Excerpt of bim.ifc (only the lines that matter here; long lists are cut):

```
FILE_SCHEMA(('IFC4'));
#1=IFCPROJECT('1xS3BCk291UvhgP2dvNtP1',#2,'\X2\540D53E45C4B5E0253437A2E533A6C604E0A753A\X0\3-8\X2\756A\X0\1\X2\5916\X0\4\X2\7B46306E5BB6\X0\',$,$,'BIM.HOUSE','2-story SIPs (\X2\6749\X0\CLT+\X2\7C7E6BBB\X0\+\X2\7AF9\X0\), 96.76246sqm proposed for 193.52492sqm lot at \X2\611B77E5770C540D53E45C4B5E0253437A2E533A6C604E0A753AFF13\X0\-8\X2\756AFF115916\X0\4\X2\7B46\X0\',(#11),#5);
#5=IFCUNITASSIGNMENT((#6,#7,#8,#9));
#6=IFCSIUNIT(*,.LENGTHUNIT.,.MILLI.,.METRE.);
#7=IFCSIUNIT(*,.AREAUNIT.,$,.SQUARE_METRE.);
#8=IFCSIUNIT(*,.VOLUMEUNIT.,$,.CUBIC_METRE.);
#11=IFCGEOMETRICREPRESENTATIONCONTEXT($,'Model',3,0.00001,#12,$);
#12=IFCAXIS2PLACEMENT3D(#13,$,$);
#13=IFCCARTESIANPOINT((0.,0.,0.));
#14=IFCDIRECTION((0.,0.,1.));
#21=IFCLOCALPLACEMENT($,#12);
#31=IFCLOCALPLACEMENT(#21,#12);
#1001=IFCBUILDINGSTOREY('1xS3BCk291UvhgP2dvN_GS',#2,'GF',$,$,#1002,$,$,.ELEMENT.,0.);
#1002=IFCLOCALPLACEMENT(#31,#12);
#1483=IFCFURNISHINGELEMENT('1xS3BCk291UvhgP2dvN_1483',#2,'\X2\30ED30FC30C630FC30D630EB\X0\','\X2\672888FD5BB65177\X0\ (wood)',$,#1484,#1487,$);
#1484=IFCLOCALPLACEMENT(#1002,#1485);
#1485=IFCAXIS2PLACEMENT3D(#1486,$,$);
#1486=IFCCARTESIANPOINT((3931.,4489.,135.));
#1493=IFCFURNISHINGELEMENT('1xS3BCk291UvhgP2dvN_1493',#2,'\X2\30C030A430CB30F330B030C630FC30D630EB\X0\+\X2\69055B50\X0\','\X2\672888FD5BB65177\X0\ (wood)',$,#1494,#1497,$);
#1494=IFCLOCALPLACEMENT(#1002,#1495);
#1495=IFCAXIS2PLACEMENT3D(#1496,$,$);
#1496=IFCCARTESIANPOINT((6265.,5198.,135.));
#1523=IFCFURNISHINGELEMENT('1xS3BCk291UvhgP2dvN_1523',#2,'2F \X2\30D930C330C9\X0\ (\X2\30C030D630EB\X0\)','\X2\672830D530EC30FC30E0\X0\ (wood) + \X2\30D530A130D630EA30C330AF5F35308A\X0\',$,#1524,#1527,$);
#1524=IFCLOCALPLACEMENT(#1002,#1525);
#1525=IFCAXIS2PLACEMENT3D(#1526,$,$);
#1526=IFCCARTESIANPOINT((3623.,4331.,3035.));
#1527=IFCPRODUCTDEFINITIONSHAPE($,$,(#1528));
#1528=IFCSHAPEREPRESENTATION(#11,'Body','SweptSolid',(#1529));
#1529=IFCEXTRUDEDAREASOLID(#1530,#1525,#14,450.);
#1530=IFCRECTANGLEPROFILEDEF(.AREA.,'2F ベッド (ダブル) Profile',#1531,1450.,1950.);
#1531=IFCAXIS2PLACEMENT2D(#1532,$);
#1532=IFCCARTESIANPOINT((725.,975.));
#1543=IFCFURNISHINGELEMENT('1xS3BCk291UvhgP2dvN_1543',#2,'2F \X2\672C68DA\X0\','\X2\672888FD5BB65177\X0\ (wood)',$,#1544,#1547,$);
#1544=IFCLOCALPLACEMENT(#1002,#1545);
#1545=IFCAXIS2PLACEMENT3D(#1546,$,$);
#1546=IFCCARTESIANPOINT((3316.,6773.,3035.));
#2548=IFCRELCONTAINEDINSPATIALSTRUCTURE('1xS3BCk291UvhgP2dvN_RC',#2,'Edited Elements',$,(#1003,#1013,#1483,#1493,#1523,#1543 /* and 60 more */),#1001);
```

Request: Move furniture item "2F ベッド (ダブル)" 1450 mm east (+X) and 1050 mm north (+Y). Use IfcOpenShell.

```python
import ifcopenshell
import ifcopenshell.api.geometry
import ifcopenshell.util.placement

model = ifcopenshell.open("bim.ifc")

item = model.by_guid("1xS3BCk291UvhgP2dvN_1523")
matrix = ifcopenshell.util.placement.get_local_placement(item.ObjectPlacement)
matrix[0, 3] += 1450.0
matrix[1, 3] += 1050.0
ifcopenshell.api.geometry.edit_object_placement(model, product=item, matrix=matrix, is_si=False)

print(ifcopenshell.util.placement.get_local_placement(item.ObjectPlacement).round(3) + 0.0)

model.write("bim-out.ifc")
```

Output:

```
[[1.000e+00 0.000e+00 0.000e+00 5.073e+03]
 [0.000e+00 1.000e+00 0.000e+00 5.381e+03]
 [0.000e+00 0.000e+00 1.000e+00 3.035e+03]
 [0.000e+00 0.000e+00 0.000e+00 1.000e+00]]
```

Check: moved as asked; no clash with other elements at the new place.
